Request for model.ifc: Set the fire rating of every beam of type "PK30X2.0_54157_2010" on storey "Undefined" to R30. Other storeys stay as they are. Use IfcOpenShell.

First a look at what the model holds.

```python
import ifcopenshell
import ifcopenshell.util.element

model = ifcopenshell.open("model.ifc")
print(model.schema)
storey = next(s for s in model.by_type("IfcBuildingStorey") if s.Name == "Undefined")
beams = [e for e in ifcopenshell.util.element.get_decomposition(storey) if e.is_a("IfcBeam")]
seen = {}
for e in beams:
    element_type = ifcopenshell.util.element.get_type(e)
    key = (element_type.Name if element_type != e and element_type else None, ifcopenshell.util.element.get_pset(e, "Pset_BeamCommon", "FireRating"))
    seen[key] = seen.get(key, 0) + 1
for (name, value), count in sorted(seen.items(), key=str):
    print(count, "x", name, "|", value)
```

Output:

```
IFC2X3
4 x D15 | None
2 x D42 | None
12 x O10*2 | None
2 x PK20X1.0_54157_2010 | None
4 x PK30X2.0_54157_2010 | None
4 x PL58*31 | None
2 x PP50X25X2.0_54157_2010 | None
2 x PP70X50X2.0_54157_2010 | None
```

```python
import ifcopenshell
import ifcopenshell.api.pset
import ifcopenshell.util.element

model = ifcopenshell.open("model.ifc")

storey = next(s for s in model.by_type("IfcBuildingStorey") if s.Name == "Undefined")
beams = [e for e in ifcopenshell.util.element.get_decomposition(storey) if e.is_a("IfcBeam")]

count = 0
for e in beams:
    element_type = ifcopenshell.util.element.get_type(e)
    if element_type in (None, e) or element_type.Name != "PK30X2.0_54157_2010":
        continue
    found = ifcopenshell.util.element.get_pset(e, "Pset_BeamCommon", should_inherit=False)
    if found:
        pset = model.by_id(found["id"])
        if len(ifcopenshell.util.element.get_elements_by_pset(pset)) > 1:
            pset = ifcopenshell.api.pset.unshare_pset(model, products=[e], pset=pset)[0]
    else:
        pset = ifcopenshell.api.pset.add_pset(model, product=e, name="Pset_BeamCommon")
    ifcopenshell.api.pset.edit_pset(model, pset=pset, properties={"FireRating": "R30"})
    count += 1

print(count, "beams updated")

model.write("model_v2.ifc")
```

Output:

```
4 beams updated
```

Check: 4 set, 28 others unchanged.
